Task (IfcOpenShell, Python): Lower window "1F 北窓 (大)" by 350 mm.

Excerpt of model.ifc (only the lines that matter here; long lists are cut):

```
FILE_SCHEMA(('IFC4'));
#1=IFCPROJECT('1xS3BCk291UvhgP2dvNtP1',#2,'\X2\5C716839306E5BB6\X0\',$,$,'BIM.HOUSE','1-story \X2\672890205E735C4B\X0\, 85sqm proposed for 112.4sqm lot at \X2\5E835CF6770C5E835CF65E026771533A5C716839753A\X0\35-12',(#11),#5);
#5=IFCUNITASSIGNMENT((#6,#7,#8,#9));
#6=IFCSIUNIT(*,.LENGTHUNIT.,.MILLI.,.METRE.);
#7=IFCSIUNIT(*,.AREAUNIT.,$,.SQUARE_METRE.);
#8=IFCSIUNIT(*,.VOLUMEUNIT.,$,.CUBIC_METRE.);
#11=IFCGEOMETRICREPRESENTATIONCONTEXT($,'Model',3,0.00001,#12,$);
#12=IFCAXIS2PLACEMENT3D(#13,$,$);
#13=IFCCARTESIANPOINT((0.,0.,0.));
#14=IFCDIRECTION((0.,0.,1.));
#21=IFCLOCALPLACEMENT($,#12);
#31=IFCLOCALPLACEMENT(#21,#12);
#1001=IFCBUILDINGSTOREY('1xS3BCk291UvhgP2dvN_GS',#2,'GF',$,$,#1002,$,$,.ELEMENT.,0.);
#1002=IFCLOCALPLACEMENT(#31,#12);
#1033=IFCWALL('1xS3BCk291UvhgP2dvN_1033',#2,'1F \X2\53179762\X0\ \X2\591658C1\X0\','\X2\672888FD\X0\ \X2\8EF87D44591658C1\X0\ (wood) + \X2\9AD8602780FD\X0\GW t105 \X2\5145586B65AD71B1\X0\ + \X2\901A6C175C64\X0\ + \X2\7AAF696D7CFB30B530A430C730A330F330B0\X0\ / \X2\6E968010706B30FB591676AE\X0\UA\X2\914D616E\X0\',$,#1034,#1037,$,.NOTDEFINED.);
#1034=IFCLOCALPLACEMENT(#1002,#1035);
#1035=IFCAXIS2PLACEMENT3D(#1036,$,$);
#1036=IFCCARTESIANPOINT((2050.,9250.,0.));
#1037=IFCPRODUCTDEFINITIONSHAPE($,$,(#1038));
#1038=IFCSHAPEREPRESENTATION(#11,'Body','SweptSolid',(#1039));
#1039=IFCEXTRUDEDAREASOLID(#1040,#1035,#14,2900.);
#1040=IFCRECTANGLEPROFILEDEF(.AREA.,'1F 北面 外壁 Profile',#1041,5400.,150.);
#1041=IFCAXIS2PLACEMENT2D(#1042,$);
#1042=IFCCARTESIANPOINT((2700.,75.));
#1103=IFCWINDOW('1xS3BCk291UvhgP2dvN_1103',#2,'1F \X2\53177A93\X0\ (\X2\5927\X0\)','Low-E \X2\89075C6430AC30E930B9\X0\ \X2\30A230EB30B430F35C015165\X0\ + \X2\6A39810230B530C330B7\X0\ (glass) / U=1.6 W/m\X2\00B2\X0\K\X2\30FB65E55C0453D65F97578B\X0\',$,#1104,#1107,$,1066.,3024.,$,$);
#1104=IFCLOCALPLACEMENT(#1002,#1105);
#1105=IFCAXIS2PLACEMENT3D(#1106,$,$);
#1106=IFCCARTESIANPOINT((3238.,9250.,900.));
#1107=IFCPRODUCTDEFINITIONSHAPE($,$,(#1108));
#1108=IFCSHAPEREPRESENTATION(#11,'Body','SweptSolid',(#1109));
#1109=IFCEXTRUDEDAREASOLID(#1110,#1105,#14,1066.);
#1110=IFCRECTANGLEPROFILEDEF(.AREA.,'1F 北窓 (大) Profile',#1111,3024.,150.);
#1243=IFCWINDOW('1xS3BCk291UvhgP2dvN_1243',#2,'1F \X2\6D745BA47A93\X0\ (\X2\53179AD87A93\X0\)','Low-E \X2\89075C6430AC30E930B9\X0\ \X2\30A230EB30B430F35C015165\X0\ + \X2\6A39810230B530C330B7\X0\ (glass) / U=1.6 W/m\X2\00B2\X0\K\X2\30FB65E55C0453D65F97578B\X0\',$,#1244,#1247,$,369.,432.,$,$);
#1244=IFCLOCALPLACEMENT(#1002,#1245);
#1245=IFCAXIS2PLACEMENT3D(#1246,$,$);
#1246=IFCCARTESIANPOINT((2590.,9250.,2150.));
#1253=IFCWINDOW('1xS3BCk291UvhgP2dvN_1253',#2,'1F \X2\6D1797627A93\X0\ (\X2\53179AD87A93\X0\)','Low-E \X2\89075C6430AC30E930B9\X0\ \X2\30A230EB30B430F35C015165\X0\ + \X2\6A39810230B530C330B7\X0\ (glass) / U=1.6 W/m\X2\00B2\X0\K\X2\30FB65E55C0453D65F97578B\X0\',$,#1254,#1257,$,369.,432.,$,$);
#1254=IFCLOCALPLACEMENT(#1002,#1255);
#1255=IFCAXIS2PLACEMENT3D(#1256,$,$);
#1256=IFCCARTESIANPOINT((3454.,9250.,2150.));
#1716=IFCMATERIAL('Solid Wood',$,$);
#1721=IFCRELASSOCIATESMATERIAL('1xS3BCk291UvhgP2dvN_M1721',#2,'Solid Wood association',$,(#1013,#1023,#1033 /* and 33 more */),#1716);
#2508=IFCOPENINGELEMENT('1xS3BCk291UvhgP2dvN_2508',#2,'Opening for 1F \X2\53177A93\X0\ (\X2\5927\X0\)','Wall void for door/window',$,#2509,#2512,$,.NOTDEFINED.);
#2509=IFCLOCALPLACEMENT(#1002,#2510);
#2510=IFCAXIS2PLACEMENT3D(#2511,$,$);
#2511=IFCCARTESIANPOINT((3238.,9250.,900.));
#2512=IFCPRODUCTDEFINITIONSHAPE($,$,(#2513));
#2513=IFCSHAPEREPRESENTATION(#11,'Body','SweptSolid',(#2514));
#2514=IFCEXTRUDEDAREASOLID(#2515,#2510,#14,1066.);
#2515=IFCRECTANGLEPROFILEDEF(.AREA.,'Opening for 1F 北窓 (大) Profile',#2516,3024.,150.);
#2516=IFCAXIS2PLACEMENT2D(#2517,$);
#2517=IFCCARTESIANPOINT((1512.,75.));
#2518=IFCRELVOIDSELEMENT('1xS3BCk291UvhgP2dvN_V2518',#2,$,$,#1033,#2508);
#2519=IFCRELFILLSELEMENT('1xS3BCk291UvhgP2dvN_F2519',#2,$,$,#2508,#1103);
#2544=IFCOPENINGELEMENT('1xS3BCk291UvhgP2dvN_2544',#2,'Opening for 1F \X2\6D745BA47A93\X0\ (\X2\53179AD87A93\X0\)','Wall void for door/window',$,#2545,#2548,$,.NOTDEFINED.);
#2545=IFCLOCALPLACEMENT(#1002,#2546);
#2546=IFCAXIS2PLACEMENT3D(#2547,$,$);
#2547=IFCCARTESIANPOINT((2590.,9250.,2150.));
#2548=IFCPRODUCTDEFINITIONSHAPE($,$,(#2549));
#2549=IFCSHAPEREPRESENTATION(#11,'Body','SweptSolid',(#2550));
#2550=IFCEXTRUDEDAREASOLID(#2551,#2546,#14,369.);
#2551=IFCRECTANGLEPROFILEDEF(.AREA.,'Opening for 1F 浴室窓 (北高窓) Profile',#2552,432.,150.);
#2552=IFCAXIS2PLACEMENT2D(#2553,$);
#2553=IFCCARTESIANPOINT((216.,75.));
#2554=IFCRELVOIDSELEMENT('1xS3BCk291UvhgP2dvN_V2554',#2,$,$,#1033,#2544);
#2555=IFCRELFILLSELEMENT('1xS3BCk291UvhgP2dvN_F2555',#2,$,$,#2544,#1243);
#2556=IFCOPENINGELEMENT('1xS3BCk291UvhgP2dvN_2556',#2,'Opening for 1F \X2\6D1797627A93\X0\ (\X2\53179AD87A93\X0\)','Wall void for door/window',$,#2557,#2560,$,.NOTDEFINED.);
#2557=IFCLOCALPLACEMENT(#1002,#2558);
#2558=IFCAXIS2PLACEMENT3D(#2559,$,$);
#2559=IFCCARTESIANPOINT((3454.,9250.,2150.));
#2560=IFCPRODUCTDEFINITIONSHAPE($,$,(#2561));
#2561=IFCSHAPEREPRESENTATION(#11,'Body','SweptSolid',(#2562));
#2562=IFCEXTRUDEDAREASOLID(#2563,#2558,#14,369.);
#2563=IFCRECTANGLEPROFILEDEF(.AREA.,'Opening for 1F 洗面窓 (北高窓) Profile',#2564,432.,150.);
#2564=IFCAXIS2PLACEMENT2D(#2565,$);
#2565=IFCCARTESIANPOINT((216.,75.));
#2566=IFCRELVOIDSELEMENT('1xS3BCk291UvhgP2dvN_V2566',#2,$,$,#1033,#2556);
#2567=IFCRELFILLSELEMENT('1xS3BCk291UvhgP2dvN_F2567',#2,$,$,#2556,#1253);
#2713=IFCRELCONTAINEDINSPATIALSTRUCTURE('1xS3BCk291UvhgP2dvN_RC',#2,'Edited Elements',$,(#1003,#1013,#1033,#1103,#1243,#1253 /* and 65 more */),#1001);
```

```python
import numpy as np
import ifcopenshell
import ifcopenshell.api.geometry
import ifcopenshell.util.placement
import ifcopenshell.util.unit

model = ifcopenshell.open("model.ifc")
unit_scale = ifcopenshell.util.unit.calculate_unit_scale(model)

window = model.by_guid("1xS3BCk291UvhgP2dvN_1103")
opening = window.FillsVoids[0].RelatingOpeningElement
dz = -0.35 / unit_scale

shift = np.array([0.0, 0.0, dz])
# The window is not placed relative to its opening, so move both.
for product in (opening, window):
    matrix = ifcopenshell.util.placement.get_local_placement(product.ObjectPlacement)
    matrix[:3, 3] += shift
    ifcopenshell.api.geometry.edit_object_placement(model, product=product, matrix=matrix, is_si=False)

print(f"moved by {dz * unit_scale:+.3f} m")

model.write("model_rev.ifc")
```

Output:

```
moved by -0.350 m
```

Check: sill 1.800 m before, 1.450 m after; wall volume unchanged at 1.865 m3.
